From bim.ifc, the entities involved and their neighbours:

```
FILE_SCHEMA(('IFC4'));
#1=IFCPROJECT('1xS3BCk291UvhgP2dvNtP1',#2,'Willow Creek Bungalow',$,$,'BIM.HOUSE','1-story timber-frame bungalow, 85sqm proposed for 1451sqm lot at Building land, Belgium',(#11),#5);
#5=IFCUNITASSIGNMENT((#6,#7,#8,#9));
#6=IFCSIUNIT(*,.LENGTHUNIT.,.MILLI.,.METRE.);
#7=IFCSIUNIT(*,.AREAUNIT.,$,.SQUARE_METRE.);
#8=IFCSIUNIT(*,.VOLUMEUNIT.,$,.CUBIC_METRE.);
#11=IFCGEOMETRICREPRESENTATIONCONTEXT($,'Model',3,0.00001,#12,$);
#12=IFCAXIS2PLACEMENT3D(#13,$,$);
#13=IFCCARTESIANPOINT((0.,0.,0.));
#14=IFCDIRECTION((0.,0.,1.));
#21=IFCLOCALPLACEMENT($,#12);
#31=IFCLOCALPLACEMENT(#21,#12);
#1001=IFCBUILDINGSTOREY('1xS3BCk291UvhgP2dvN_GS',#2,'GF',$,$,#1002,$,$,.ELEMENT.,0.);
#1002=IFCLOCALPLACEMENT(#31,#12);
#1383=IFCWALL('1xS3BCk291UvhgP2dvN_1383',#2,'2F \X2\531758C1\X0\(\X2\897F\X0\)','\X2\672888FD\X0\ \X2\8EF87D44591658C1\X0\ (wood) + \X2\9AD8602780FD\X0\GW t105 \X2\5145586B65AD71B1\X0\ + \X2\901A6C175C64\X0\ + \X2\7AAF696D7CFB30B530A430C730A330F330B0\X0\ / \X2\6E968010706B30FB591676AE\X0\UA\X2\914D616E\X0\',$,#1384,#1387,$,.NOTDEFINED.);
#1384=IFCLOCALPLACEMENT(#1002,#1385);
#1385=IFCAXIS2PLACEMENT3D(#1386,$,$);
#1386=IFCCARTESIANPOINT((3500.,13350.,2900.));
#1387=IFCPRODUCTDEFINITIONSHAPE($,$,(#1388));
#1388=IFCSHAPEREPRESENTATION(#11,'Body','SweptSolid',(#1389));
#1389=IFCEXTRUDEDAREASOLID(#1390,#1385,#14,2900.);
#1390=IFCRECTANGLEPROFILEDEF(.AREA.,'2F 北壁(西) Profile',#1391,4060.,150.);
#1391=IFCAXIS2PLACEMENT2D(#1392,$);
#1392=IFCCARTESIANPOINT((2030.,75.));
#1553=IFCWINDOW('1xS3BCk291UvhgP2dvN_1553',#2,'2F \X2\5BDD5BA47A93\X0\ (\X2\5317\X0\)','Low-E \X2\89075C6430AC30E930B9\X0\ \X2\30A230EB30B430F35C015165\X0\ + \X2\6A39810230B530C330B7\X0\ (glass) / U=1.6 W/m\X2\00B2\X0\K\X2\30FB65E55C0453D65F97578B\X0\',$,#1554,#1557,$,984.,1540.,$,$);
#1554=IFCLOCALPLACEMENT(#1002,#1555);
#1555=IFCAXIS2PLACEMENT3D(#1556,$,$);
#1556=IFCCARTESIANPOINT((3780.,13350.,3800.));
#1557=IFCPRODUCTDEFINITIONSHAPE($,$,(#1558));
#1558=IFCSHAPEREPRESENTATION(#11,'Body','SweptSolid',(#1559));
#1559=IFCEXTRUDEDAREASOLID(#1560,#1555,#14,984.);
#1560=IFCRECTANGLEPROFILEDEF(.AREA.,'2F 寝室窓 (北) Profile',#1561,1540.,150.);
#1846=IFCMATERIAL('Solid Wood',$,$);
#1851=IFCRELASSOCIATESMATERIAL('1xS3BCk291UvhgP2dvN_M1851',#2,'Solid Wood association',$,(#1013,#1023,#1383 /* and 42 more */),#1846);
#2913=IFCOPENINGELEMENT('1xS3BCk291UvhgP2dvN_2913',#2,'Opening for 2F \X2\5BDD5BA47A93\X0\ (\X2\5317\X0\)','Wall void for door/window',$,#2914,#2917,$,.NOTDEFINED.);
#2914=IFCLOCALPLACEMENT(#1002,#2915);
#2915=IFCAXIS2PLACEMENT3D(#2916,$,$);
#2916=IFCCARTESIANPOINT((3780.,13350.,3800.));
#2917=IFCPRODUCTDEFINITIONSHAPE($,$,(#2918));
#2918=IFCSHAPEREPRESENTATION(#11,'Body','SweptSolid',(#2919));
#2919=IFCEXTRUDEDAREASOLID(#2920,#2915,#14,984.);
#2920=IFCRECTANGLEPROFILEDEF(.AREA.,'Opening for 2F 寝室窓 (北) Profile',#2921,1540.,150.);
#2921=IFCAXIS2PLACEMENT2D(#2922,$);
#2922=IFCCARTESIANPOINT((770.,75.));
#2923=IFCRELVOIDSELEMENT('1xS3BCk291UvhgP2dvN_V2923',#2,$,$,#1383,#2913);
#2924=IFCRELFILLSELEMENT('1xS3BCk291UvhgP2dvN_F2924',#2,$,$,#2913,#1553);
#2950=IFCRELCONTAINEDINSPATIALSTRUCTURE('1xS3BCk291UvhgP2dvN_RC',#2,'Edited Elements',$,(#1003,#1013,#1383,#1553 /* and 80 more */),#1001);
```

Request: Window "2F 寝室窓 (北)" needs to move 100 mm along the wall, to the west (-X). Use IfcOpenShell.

```python
import ifcopenshell
import ifcopenshell.api.geometry
import ifcopenshell.util.placement
import ifcopenshell.util.unit

model = ifcopenshell.open("bim.ifc")
unit_scale = ifcopenshell.util.unit.calculate_unit_scale(model)

window = model.by_guid("1xS3BCk291UvhgP2dvN_1553")
opening = window.FillsVoids[0].RelatingOpeningElement
wall = opening.VoidsElements[0].RelatingBuildingElement

wall_matrix = ifcopenshell.util.placement.get_local_placement(wall.ObjectPlacement)
shift = wall_matrix[:3, 0] * -0.1 / unit_scale
before = ifcopenshell.util.placement.get_local_placement(window.ObjectPlacement)[:3, 3].copy()

# The window is not placed relative to its opening, so move both.
for product in (opening, window):
    matrix = ifcopenshell.util.placement.get_local_placement(product.ObjectPlacement)
    matrix[:3, 3] += shift
    ifcopenshell.api.geometry.edit_object_placement(model, product=product, matrix=matrix, is_si=False)

after = ifcopenshell.util.placement.get_local_placement(window.ObjectPlacement)[:3, 3]
print("window moved by", (after - before).round(3) + 0.0)

model.write("bim_edited.ifc")
```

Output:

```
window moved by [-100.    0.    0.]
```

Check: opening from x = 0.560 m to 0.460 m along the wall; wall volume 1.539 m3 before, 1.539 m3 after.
